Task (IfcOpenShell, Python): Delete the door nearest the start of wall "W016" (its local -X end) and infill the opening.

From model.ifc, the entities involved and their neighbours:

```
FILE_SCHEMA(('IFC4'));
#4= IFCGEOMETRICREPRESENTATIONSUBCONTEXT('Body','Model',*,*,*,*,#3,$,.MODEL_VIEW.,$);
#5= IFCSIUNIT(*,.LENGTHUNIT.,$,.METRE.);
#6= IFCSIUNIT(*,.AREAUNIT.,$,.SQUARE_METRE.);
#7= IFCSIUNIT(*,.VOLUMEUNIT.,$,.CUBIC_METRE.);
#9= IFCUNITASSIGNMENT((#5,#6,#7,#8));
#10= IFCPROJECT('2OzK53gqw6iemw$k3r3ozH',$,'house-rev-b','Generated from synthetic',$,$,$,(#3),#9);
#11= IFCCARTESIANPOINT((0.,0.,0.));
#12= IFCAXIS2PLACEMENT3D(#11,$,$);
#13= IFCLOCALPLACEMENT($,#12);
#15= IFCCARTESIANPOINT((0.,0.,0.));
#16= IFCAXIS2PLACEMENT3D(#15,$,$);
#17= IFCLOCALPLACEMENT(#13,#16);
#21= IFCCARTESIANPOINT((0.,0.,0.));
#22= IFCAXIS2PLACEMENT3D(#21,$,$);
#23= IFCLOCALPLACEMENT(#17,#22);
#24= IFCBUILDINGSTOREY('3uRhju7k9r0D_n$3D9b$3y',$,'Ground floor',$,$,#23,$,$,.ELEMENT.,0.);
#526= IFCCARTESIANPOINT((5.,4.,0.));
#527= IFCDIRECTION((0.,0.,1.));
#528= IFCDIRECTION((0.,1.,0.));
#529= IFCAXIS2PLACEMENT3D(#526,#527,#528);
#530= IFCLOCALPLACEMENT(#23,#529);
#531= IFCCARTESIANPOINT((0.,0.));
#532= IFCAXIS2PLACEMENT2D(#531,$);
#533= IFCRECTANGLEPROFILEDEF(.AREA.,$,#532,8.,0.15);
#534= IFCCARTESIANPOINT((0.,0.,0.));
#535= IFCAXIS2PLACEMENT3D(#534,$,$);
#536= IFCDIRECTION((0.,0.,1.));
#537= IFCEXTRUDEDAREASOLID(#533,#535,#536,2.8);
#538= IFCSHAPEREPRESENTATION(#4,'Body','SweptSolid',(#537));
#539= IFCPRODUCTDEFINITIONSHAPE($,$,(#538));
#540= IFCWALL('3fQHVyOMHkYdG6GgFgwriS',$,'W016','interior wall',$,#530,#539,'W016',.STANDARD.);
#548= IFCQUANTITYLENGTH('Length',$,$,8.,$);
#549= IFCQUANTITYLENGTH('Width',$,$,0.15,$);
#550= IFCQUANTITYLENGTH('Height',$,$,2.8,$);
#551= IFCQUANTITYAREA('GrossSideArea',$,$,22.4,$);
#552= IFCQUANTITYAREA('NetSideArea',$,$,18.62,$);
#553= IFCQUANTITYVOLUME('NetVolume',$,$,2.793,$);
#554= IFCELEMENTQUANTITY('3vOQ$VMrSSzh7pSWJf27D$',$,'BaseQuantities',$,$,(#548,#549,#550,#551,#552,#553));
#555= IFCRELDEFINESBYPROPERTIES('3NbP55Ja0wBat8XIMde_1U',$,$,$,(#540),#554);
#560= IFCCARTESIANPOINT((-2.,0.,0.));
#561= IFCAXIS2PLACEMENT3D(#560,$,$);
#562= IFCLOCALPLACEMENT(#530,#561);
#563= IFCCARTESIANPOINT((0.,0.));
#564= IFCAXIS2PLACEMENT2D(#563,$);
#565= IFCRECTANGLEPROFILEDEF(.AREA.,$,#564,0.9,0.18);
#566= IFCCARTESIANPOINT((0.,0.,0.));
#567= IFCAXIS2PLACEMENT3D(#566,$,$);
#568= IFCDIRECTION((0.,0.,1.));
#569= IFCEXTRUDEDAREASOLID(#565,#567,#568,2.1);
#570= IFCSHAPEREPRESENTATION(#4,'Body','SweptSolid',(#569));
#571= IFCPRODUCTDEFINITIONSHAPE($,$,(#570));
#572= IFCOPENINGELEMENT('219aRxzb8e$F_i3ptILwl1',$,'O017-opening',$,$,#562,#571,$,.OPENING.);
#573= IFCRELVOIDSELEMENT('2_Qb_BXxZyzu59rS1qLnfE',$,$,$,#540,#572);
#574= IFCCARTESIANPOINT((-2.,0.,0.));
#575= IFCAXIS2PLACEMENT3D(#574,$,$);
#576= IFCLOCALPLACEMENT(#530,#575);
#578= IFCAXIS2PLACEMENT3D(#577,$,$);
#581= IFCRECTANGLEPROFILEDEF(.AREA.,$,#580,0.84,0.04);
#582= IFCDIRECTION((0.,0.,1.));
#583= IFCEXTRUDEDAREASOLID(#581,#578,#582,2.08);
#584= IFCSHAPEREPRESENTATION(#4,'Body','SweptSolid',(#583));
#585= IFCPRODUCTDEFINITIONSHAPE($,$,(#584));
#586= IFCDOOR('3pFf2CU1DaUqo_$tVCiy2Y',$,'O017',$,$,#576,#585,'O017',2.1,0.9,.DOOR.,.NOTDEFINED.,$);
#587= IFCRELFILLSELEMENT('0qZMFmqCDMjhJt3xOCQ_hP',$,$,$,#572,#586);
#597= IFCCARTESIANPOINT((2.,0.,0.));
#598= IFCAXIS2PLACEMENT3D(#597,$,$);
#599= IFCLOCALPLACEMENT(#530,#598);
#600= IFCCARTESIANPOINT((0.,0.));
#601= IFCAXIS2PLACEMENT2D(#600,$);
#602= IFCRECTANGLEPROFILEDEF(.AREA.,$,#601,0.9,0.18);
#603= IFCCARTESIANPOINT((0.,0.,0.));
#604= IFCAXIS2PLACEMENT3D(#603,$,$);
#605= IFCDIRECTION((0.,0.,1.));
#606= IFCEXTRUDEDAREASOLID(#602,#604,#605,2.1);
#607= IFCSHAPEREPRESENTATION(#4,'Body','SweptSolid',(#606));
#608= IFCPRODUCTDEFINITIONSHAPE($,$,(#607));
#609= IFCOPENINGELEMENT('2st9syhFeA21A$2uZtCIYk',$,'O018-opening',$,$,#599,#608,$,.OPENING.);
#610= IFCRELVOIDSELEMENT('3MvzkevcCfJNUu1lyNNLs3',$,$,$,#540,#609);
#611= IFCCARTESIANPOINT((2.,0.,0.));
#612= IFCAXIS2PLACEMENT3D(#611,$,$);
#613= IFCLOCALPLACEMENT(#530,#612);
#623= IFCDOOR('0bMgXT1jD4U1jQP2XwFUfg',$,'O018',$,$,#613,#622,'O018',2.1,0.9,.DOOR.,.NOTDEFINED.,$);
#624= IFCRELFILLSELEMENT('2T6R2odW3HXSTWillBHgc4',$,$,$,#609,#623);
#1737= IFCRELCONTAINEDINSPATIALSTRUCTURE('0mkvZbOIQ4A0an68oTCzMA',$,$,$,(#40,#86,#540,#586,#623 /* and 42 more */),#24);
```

```python
import ifcopenshell
import ifcopenshell.api.feature
import ifcopenshell.api.pset
import ifcopenshell.api.root
import ifcopenshell.geom
import ifcopenshell.util.element
import ifcopenshell.util.shape
import ifcopenshell.util.unit

model = ifcopenshell.open("model.ifc")
area_scale = ifcopenshell.util.unit.calculate_unit_scale(model, "AREAUNIT")
volume_scale = ifcopenshell.util.unit.calculate_unit_scale(model, "VOLUMEUNIT")
settings = ifcopenshell.geom.settings()


def volume(element):
    """Net volume in cubic metres, openings subtracted."""
    shape = ifcopenshell.geom.create_shape(settings, element)
    return ifcopenshell.util.shape.get_volume(shape.geometry)


door = model.by_guid("3pFf2CU1DaUqo_$tVCiy2Y")
opening = door.FillsVoids[0].RelatingOpeningElement
wall = opening.VoidsElements[0].RelatingBuildingElement
before = volume(wall)

ifcopenshell.api.root.remove_product(model, product=door)
ifcopenshell.api.feature.remove_feature(model, feature=opening)

after = volume(wall)
thickness = 0.15  # wall thickness in metres

# Update the wall's stored quantities.
qto = model.by_id(ifcopenshell.util.element.get_pset(wall, "BaseQuantities", should_inherit=False)["id"])
ifcopenshell.api.pset.edit_qto(model, qto=qto, properties={
    "NetSideArea": after / thickness / area_scale,
    "NetVolume": after / volume_scale,
})

print(f"wall volume {before:.3f} -> {after:.3f} m3")

model.write("model-out.ifc")
```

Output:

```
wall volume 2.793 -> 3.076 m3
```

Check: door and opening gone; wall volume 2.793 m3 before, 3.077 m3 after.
